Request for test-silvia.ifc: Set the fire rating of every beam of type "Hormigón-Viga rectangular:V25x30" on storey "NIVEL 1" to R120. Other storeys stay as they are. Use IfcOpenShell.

First a look at what the model holds.

```python
import ifcopenshell
import ifcopenshell.util.element

model = ifcopenshell.open("test-silvia.ifc")
print(model.schema)
storey = next(s for s in model.by_type("IfcBuildingStorey") if s.Name == "NIVEL 1")
beams = [e for e in ifcopenshell.util.element.get_decomposition(storey) if e.is_a("IfcBeam")]
seen = {}
for e in beams:
    element_type = ifcopenshell.util.element.get_type(e)
    key = (element_type.Name if element_type != e and element_type else None, ifcopenshell.util.element.get_pset(e, "Pset_BeamCommon", "FireRating"))
    seen[key] = seen.get(key, 0) + 1
for (name, value), count in sorted(seen.items(), key=str):
    print(count, "x", name, "|", value)
```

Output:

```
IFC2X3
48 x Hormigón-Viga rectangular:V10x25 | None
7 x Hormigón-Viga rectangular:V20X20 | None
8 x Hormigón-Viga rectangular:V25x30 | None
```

```python
import ifcopenshell
import ifcopenshell.api.pset
import ifcopenshell.util.element

model = ifcopenshell.open("test-silvia.ifc")

storey = next(s for s in model.by_type("IfcBuildingStorey") if s.Name == "NIVEL 1")
beams = [e for e in ifcopenshell.util.element.get_decomposition(storey) if e.is_a("IfcBeam")]

count = 0
for e in beams:
    element_type = ifcopenshell.util.element.get_type(e)
    if element_type in (None, e) or element_type.Name != "Hormigón-Viga rectangular:V25x30":
        continue
    # add_pset returns the element's existing set when there is one.
    pset = ifcopenshell.api.pset.add_pset(model, product=e, name="Pset_BeamCommon")
    ifcopenshell.api.pset.edit_pset(model, pset=pset, properties={"FireRating": "R120"})
    count += 1

print(count, "beams updated")

model.write("test-silvia_edited.ifc")
```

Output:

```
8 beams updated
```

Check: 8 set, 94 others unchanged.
